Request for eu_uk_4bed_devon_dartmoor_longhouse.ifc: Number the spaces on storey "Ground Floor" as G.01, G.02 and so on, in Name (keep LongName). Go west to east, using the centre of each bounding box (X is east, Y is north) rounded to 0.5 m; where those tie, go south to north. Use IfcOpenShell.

First a look at what the model holds.

```python
import ifcopenshell
import ifcopenshell.util.element
import ifcopenshell.util.placement

model = ifcopenshell.open("eu_uk_4bed_devon_dartmoor_longhouse.ifc")
print(model.schema)
storey = next(s for s in model.by_type("IfcBuildingStorey") if s.Name == "Ground Floor")
spaces = [e for e in ifcopenshell.util.element.get_decomposition(storey) if e.is_a("IfcSpace")]
for e in sorted(spaces, key=lambda e: e.id()):
    origin = ifcopenshell.util.placement.get_local_placement(e.ObjectPlacement)[:3, 3]
    print(e.id(), e.Name, e.LongName, origin.round(2) + 0.0, sep=" | ")
```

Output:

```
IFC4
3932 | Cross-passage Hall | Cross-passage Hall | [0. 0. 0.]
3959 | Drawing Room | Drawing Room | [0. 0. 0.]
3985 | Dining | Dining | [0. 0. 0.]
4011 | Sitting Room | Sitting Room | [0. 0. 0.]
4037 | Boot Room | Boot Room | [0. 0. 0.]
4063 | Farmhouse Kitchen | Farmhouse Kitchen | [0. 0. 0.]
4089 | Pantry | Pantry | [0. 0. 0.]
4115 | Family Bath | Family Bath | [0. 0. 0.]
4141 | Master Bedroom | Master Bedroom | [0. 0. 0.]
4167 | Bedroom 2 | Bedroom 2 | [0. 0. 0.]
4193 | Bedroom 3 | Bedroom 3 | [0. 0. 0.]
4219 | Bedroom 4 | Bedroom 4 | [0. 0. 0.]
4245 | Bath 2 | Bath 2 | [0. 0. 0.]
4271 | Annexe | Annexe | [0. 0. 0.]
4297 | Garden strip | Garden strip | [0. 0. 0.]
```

```python
import ifcopenshell
import ifcopenshell.geom
import ifcopenshell.util.element
import ifcopenshell.util.shape

model = ifcopenshell.open("eu_uk_4bed_devon_dartmoor_longhouse.ifc")
settings = ifcopenshell.geom.settings()
settings.set("use-world-coords", True)


def centre(element):
    shape = ifcopenshell.geom.create_shape(settings, element)
    return ifcopenshell.util.shape.get_bbox_centroid(shape.geometry)


storey = next(s for s in model.by_type("IfcBuildingStorey") if s.Name == "Ground Floor")
spaces = [e for e in ifcopenshell.util.element.get_decomposition(storey) if e.is_a("IfcSpace")]

# Insertion points can sit at a corner or the storey origin, so sort by the geometry (in metres).
centres = {e: centre(e) for e in spaces}
spaces.sort(key=lambda e: (round(centres[e][0] / 0.5), centres[e][1]))

for i, e in enumerate(spaces, start=1):
    number = f"G.{i:02d}"
    e.Name = number
    print(e.id(), number)

model.write("eu_uk_4bed_devon_dartmoor_longhouse_rev.ifc")
```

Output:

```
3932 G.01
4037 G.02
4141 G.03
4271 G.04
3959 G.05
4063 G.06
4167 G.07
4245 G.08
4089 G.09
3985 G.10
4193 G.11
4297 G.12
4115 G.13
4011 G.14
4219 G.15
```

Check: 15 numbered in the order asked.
